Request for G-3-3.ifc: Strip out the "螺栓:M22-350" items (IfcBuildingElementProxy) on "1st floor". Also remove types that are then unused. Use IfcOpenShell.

First a look at what the model holds.

```python
import ifcopenshell
import ifcopenshell.util.element

model = ifcopenshell.open("G-3-3.ifc")
print(model.schema)
storey = next(s for s in model.by_type("IfcBuildingStorey") if s.Name == "1st floor")
proxies = [e for e in ifcopenshell.util.element.get_decomposition(storey) if e.is_a("IfcBuildingElementProxy")]
seen = {}
for e in proxies:
    element_type = ifcopenshell.util.element.get_type(e)
    name = element_type.Name if element_type not in (None, e) else None
    seen[name] = seen.get(name, 0) + 1
for name, count in sorted(seen.items(), key=str):
    print(count, "x", name)
```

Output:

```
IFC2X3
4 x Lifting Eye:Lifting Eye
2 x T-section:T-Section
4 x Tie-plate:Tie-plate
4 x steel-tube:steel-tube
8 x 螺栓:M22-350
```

```python
import ifcopenshell
import ifcopenshell.api.root
import ifcopenshell.util.element

model = ifcopenshell.open("G-3-3.ifc")

storey = next(s for s in model.by_type("IfcBuildingStorey") if s.Name == "1st floor")
proxies = [e for e in ifcopenshell.util.element.get_decomposition(storey) if e.is_a("IfcBuildingElementProxy")]
targets = [e for e in proxies if (t := ifcopenshell.util.element.get_type(e)) not in (None, e) and t.Name == "螺栓:M22-350"]
types = {ifcopenshell.util.element.get_type(e) for e in targets} - {None, *targets}

for e in targets:
    ifcopenshell.api.root.remove_product(model, product=e)
print(len(targets), "removed")

unused = [t for t in types if not ifcopenshell.util.element.get_types(t)]
for t in unused:
    ifcopenshell.api.root.remove_product(model, product=t)
print(len(unused), "unused types removed")

model.write("G-3-3-out.ifc")
```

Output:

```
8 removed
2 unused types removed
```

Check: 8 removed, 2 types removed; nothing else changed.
